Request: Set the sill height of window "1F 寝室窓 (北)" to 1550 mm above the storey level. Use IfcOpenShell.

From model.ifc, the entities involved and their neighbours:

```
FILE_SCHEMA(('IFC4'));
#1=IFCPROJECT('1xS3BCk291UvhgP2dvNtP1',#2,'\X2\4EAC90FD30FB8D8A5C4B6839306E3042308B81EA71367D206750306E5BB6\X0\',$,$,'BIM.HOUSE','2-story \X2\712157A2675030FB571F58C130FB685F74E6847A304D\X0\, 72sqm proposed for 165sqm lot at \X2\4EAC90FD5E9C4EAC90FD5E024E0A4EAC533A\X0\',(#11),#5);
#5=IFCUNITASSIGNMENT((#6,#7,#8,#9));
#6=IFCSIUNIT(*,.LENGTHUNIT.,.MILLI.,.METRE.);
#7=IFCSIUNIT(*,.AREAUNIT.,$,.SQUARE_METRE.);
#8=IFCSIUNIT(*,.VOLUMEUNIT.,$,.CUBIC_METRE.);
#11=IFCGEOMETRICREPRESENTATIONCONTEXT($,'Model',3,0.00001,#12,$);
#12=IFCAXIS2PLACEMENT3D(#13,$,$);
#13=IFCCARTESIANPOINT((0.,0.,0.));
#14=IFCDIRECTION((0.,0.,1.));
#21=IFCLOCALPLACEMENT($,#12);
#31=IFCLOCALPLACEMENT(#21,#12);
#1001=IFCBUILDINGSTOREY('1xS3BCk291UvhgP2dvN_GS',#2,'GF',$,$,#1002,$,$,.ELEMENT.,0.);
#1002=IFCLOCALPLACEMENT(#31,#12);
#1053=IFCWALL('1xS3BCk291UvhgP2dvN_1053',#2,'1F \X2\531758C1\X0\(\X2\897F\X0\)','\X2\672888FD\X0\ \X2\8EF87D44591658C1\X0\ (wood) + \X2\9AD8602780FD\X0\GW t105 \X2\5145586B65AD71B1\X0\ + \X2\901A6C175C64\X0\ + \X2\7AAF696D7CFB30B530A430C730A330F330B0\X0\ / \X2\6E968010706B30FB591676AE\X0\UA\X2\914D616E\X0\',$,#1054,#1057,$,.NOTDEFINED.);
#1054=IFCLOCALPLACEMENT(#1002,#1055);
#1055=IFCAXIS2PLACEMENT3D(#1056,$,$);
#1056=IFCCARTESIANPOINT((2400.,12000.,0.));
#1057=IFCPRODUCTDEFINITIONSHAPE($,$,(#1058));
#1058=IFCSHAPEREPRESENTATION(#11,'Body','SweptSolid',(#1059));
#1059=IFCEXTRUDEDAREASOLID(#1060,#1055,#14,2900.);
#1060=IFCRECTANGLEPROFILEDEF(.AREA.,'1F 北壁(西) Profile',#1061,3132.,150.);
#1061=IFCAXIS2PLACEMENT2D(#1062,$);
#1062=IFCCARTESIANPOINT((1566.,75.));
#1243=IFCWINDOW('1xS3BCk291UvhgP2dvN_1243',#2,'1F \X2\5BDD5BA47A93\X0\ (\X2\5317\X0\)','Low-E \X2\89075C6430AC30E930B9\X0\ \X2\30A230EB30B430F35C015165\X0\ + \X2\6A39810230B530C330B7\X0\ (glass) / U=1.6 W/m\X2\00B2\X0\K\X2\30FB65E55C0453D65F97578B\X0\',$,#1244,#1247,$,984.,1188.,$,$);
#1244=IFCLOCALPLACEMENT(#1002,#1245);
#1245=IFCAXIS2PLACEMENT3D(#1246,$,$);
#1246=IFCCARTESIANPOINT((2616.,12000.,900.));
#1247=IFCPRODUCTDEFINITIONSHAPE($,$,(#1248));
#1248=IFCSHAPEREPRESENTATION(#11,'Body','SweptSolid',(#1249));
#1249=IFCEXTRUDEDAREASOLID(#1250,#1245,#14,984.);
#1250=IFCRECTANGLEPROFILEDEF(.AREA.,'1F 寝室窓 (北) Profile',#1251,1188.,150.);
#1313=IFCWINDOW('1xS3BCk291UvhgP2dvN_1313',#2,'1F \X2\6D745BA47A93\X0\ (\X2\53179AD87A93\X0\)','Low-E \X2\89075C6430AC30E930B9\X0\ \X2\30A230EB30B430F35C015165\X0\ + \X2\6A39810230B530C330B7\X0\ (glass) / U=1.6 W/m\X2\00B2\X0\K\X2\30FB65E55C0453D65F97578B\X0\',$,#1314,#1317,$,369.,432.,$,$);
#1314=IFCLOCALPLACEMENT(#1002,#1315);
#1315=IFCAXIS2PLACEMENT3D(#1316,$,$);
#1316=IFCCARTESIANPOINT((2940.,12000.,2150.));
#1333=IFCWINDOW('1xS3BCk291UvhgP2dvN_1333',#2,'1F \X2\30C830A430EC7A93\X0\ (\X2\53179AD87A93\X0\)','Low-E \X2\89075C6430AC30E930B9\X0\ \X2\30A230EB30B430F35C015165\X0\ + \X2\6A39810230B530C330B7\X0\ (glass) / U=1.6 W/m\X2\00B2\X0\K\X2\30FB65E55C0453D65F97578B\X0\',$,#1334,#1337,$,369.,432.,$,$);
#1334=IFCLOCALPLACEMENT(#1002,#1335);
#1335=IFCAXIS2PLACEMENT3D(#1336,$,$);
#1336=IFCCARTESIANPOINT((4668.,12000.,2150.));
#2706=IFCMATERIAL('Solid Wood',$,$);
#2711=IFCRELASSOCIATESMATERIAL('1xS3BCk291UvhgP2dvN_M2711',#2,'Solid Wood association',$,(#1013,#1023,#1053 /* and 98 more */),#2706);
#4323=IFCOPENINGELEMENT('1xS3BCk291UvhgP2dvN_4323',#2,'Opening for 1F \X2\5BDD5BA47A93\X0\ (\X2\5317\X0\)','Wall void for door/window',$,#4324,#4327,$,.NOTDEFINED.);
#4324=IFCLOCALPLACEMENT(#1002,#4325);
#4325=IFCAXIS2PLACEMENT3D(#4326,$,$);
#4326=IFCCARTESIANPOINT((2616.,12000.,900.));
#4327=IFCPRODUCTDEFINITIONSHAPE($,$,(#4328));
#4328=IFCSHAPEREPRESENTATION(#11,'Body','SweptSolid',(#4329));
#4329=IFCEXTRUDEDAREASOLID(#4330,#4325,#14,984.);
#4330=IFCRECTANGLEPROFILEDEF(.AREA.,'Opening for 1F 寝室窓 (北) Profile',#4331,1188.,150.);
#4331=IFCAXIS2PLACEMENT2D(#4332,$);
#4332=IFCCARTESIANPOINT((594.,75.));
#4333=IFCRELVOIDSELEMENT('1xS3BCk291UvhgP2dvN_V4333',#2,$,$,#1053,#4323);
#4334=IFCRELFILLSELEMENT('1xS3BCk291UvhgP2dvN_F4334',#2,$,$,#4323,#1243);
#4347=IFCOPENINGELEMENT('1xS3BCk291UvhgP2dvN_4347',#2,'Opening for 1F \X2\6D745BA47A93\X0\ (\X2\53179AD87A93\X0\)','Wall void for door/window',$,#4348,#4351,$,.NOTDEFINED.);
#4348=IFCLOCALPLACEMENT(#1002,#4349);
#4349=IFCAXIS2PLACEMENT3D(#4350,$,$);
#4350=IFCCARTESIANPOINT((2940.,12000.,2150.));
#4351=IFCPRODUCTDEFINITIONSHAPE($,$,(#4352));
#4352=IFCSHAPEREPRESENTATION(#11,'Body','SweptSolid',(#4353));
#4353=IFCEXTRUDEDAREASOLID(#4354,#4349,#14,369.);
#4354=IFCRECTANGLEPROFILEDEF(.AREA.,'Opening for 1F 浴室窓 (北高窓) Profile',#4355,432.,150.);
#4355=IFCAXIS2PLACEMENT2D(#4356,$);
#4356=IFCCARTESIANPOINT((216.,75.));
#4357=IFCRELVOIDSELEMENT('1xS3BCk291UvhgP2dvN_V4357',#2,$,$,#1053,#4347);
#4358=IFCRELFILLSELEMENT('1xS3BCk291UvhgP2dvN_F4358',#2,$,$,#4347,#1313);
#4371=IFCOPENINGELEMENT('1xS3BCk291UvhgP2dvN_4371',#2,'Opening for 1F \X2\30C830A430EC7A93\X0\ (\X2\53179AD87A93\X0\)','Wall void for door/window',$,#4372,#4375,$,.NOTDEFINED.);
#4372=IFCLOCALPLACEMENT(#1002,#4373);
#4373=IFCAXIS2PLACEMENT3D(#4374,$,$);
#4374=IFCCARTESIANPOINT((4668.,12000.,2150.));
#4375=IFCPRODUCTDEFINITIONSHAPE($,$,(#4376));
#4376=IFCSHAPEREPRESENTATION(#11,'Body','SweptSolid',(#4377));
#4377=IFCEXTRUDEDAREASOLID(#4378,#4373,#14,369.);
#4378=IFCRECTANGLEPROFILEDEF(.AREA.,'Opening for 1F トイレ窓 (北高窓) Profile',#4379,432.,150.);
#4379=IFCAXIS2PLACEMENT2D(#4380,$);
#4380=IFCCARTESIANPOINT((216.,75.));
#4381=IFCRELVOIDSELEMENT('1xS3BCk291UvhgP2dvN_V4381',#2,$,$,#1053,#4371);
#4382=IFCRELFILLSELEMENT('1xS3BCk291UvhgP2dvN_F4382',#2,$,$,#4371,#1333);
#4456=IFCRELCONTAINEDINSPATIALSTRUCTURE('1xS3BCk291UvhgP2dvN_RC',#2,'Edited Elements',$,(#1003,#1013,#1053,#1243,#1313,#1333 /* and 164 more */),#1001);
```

```python
import numpy as np
import ifcopenshell
import ifcopenshell.api.geometry
import ifcopenshell.geom
import ifcopenshell.util.element
import ifcopenshell.util.placement
import ifcopenshell.util.shape
import ifcopenshell.util.unit

model = ifcopenshell.open("model.ifc")
unit_scale = ifcopenshell.util.unit.calculate_unit_scale(model)

window = model.by_id(1243)
opening = window.FillsVoids[0].RelatingOpeningElement
storey = ifcopenshell.util.element.get_container(window, ifc_class="IfcBuildingStorey")
level = ifcopenshell.util.placement.get_local_placement(storey.ObjectPlacement)[2, 3]

# The opening's origin need not be at the sill, so measure its lowest point.
shape = ifcopenshell.geom.create_shape(ifcopenshell.geom.settings(), opening)
bottom = ifcopenshell.util.shape.get_shape_bottom_elevation(shape, shape.geometry) / unit_scale
dz = level + 1.55 / unit_scale - bottom

shift = np.array([0.0, 0.0, dz])
# The window is not placed relative to its opening, so move both.
for product in (opening, window):
    matrix = ifcopenshell.util.placement.get_local_placement(product.ObjectPlacement)
    matrix[:3, 3] += shift
    ifcopenshell.api.geometry.edit_object_placement(model, product=product, matrix=matrix, is_si=False)

print(f"moved by {dz * unit_scale:+.3f} m")

model.write("model-out.ifc")
```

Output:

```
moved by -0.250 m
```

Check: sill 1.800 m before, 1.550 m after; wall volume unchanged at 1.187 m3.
